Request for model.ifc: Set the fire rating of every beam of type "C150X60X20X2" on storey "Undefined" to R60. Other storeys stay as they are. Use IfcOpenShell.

First a look at what the model holds.

```python
import ifcopenshell
import ifcopenshell.util.element

model = ifcopenshell.open("model.ifc")
print(model.schema)
storey = next(s for s in model.by_type("IfcBuildingStorey") if s.Name == "Undefined")
beams = [e for e in ifcopenshell.util.element.get_decomposition(storey) if e.is_a("IfcBeam")]
seen = {}
for e in beams:
    element_type = ifcopenshell.util.element.get_type(e)
    key = (element_type.Name if element_type != e and element_type else None, ifcopenshell.util.element.get_pset(e, "Pset_BeamCommon", "FireRating"))
    seen[key] = seen.get(key, 0) + 1
for (name, value), count in sorted(seen.items(), key=str):
    print(count, "x", name, "|", value)
```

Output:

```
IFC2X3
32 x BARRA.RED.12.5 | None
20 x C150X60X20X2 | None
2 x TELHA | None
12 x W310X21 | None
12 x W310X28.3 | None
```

```python
import ifcopenshell
import ifcopenshell.api.pset
import ifcopenshell.util.element

model = ifcopenshell.open("model.ifc")

storey = next(s for s in model.by_type("IfcBuildingStorey") if s.Name == "Undefined")
beams = [e for e in ifcopenshell.util.element.get_decomposition(storey) if e.is_a("IfcBeam")]

count = 0
for e in beams:
    element_type = ifcopenshell.util.element.get_type(e)
    if element_type in (None, e) or element_type.Name != "C150X60X20X2":
        continue
    found = ifcopenshell.util.element.get_pset(e, "Pset_BeamCommon", should_inherit=False)
    if found:
        pset = model.by_id(found["id"])
        if len(ifcopenshell.util.element.get_elements_by_pset(pset)) > 1:
            pset = ifcopenshell.api.pset.unshare_pset(model, products=[e], pset=pset)[0]
    else:
        pset = ifcopenshell.api.pset.add_pset(model, product=e, name="Pset_BeamCommon")
    ifcopenshell.api.pset.edit_pset(model, pset=pset, properties={"FireRating": "R60"})
    count += 1

print(count, "beams updated")

model.write("model_v2.ifc")
```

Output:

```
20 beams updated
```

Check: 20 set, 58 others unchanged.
